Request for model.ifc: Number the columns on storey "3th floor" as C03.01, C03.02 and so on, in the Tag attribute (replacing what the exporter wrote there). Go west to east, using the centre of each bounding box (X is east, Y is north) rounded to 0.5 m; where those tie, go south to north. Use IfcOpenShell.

First a look at what the model holds.

```python
import ifcopenshell
import ifcopenshell.util.element
import ifcopenshell.util.placement

model = ifcopenshell.open("model.ifc")
print(model.schema)
storey = next(s for s in model.by_type("IfcBuildingStorey") if s.Name == "3th floor")
columns = [e for e in ifcopenshell.util.element.get_decomposition(storey) if e.is_a("IfcColumn")]
for e in sorted(columns, key=lambda e: e.id()):
    origin = ifcopenshell.util.placement.get_local_placement(e.ObjectPlacement)[:3, 3]
    print(e.id(), e.Tag, e.Name, origin.round(2) + 0.0, sep=" | ")
```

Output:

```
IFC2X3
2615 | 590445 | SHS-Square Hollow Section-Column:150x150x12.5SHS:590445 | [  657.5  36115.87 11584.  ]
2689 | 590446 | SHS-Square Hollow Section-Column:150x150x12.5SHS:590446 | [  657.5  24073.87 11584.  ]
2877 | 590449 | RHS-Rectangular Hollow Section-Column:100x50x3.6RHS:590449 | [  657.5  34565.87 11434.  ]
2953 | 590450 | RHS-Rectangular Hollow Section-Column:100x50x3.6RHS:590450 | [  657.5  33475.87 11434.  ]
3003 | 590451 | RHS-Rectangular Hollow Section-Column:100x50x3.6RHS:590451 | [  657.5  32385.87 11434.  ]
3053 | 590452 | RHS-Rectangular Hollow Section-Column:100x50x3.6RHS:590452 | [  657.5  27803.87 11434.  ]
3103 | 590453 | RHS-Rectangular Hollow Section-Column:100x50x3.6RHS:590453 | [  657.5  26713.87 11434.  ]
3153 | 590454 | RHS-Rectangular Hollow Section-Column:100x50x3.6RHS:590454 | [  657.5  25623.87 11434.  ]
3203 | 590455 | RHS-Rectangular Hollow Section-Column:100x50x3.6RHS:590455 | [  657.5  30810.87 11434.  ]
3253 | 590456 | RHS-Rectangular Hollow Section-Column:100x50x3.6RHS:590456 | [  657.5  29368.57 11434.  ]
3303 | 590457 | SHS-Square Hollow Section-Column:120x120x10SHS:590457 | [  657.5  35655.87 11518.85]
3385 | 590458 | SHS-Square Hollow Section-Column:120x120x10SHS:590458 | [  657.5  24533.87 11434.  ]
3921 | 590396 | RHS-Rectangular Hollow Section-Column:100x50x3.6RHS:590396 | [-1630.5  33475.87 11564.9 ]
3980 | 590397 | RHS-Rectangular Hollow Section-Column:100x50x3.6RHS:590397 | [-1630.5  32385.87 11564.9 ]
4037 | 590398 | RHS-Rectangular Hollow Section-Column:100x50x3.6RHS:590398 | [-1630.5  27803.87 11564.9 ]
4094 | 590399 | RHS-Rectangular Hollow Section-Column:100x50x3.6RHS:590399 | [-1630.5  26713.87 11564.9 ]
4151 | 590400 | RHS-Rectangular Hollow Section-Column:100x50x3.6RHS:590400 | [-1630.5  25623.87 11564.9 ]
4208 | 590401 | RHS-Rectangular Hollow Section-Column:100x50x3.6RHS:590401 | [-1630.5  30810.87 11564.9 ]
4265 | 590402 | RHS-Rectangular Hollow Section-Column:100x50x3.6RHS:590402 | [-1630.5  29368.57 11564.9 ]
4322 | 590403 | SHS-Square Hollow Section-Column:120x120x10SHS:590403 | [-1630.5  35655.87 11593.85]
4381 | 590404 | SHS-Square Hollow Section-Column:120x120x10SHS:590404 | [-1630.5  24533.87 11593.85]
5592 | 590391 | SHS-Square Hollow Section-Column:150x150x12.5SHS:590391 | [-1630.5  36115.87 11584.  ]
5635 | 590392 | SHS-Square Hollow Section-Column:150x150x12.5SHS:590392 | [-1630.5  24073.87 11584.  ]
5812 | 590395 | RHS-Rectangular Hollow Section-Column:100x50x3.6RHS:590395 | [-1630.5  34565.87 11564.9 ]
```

```python
import ifcopenshell
import ifcopenshell.geom
import ifcopenshell.util.element
import ifcopenshell.util.shape

model = ifcopenshell.open("model.ifc")
settings = ifcopenshell.geom.settings()
settings.set("use-world-coords", True)


def centre(element):
    shape = ifcopenshell.geom.create_shape(settings, element)
    return ifcopenshell.util.shape.get_bbox_centroid(shape.geometry)


storey = next(s for s in model.by_type("IfcBuildingStorey") if s.Name == "3th floor")
columns = [e for e in ifcopenshell.util.element.get_decomposition(storey) if e.is_a("IfcColumn")]

# Insertion points can sit at a corner or the storey origin, so sort by the geometry (in metres).
centres = {e: centre(e) for e in columns}
columns.sort(key=lambda e: (round(centres[e][0] / 0.5), centres[e][1]))

for i, e in enumerate(columns, start=1):
    number = f"C03.{i:02d}"
    e.Tag = number
    print(e.id(), number)

model.write("model_edited.ifc")
```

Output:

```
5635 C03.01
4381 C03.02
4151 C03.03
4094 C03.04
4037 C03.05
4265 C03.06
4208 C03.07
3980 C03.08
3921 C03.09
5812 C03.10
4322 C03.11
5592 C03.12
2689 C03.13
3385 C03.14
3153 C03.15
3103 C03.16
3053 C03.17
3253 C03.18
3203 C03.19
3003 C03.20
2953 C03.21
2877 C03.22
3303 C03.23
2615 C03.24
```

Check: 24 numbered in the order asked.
